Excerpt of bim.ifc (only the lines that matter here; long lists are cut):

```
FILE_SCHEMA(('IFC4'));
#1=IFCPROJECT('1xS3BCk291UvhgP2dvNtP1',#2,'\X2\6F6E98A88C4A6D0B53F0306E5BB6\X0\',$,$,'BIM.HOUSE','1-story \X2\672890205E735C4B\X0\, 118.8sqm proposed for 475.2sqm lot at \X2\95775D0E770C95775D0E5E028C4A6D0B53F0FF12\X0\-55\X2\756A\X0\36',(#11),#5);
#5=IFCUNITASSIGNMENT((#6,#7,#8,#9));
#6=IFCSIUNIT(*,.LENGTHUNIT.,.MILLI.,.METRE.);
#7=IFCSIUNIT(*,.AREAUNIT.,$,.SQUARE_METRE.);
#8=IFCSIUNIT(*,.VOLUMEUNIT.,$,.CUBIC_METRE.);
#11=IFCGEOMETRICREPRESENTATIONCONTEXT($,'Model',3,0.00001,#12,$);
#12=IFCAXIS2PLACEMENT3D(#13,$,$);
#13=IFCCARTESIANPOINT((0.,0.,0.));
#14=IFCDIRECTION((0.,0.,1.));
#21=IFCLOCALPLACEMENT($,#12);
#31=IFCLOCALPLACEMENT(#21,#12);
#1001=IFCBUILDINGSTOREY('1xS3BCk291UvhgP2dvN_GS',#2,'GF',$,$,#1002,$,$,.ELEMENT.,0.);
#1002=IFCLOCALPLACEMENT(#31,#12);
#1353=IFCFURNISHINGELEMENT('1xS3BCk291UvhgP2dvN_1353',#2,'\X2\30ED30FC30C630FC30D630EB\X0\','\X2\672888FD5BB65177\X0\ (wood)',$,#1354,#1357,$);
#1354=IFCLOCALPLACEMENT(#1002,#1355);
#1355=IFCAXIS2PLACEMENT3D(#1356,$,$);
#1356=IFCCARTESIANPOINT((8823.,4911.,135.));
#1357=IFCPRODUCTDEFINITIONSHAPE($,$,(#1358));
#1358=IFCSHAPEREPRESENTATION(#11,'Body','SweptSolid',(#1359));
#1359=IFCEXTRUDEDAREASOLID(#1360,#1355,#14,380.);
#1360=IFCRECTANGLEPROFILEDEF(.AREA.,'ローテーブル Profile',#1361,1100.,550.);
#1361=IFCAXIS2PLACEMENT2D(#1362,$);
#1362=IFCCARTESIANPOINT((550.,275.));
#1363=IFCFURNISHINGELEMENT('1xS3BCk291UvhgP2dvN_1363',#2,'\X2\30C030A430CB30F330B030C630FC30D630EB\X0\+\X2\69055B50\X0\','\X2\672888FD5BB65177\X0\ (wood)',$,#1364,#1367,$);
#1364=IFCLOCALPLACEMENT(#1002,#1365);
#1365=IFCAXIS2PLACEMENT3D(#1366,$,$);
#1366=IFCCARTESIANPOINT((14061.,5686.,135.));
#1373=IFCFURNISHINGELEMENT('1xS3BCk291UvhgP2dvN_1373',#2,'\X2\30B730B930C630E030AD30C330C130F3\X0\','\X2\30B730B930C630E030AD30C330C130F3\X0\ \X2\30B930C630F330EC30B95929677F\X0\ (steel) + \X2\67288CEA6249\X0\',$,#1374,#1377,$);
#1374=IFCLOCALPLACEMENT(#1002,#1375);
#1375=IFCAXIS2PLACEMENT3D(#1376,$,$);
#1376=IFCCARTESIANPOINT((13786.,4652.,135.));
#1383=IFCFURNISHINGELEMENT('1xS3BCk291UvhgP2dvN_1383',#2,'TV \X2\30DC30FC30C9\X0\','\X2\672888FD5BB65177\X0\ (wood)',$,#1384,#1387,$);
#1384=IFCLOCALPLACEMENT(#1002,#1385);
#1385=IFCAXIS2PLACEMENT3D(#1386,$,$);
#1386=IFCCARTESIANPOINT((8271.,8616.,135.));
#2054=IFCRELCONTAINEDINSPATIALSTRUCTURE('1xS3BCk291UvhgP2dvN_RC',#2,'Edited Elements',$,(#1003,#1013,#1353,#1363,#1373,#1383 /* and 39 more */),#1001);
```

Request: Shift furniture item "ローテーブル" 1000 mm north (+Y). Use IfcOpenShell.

```python
import ifcopenshell
import ifcopenshell.api.geometry
import ifcopenshell.util.placement

model = ifcopenshell.open("bim.ifc")

item = model.by_id(1353)
matrix = ifcopenshell.util.placement.get_local_placement(item.ObjectPlacement)
matrix[1, 3] += 1000.0
ifcopenshell.api.geometry.edit_object_placement(model, product=item, matrix=matrix, is_si=False)

print(ifcopenshell.util.placement.get_local_placement(item.ObjectPlacement).round(3) + 0.0)

model.write("bim_rev.ifc")
```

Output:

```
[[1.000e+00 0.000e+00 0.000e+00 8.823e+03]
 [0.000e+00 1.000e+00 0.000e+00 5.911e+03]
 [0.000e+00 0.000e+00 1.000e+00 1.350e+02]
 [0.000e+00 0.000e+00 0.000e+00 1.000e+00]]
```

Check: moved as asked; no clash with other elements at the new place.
